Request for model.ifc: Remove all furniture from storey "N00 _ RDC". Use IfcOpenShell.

First a look at what the model holds.

```python
import ifcopenshell
import ifcopenshell.util.element

model = ifcopenshell.open("model.ifc")
print(model.schema)
storey = next(s for s in model.by_type("IfcBuildingStorey") if s.Name == "N00 _ RDC")
furniture = [e for e in ifcopenshell.util.element.get_decomposition(storey) if e.is_a("IfcFurnishingElement")]
seen = {}
for e in furniture:
    element_type = ifcopenshell.util.element.get_type(e)
    name = element_type.Name if element_type not in (None, e) else None
    seen[name] = seen.get(name, 0) + 1
for name, count in sorted(seen.items(), key=str):
    print(count, "x", name)
```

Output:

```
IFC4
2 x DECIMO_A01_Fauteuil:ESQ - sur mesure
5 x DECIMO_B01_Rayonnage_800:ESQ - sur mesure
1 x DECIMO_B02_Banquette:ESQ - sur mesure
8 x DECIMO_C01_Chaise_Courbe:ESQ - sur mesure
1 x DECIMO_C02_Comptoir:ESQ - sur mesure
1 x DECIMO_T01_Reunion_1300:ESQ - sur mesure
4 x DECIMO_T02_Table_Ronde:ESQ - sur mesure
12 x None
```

```python
import ifcopenshell
import ifcopenshell.api.root
import ifcopenshell.util.element

model = ifcopenshell.open("model.ifc")

storey = next(s for s in model.by_type("IfcBuildingStorey") if s.Name == "N00 _ RDC")
furniture = [e for e in ifcopenshell.util.element.get_decomposition(storey) if e.is_a("IfcFurnishingElement")]

for e in furniture:
    ifcopenshell.api.root.remove_product(model, product=e)
print(len(furniture), "removed")

model.write("model_updated.ifc")
```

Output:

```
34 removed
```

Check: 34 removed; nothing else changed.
